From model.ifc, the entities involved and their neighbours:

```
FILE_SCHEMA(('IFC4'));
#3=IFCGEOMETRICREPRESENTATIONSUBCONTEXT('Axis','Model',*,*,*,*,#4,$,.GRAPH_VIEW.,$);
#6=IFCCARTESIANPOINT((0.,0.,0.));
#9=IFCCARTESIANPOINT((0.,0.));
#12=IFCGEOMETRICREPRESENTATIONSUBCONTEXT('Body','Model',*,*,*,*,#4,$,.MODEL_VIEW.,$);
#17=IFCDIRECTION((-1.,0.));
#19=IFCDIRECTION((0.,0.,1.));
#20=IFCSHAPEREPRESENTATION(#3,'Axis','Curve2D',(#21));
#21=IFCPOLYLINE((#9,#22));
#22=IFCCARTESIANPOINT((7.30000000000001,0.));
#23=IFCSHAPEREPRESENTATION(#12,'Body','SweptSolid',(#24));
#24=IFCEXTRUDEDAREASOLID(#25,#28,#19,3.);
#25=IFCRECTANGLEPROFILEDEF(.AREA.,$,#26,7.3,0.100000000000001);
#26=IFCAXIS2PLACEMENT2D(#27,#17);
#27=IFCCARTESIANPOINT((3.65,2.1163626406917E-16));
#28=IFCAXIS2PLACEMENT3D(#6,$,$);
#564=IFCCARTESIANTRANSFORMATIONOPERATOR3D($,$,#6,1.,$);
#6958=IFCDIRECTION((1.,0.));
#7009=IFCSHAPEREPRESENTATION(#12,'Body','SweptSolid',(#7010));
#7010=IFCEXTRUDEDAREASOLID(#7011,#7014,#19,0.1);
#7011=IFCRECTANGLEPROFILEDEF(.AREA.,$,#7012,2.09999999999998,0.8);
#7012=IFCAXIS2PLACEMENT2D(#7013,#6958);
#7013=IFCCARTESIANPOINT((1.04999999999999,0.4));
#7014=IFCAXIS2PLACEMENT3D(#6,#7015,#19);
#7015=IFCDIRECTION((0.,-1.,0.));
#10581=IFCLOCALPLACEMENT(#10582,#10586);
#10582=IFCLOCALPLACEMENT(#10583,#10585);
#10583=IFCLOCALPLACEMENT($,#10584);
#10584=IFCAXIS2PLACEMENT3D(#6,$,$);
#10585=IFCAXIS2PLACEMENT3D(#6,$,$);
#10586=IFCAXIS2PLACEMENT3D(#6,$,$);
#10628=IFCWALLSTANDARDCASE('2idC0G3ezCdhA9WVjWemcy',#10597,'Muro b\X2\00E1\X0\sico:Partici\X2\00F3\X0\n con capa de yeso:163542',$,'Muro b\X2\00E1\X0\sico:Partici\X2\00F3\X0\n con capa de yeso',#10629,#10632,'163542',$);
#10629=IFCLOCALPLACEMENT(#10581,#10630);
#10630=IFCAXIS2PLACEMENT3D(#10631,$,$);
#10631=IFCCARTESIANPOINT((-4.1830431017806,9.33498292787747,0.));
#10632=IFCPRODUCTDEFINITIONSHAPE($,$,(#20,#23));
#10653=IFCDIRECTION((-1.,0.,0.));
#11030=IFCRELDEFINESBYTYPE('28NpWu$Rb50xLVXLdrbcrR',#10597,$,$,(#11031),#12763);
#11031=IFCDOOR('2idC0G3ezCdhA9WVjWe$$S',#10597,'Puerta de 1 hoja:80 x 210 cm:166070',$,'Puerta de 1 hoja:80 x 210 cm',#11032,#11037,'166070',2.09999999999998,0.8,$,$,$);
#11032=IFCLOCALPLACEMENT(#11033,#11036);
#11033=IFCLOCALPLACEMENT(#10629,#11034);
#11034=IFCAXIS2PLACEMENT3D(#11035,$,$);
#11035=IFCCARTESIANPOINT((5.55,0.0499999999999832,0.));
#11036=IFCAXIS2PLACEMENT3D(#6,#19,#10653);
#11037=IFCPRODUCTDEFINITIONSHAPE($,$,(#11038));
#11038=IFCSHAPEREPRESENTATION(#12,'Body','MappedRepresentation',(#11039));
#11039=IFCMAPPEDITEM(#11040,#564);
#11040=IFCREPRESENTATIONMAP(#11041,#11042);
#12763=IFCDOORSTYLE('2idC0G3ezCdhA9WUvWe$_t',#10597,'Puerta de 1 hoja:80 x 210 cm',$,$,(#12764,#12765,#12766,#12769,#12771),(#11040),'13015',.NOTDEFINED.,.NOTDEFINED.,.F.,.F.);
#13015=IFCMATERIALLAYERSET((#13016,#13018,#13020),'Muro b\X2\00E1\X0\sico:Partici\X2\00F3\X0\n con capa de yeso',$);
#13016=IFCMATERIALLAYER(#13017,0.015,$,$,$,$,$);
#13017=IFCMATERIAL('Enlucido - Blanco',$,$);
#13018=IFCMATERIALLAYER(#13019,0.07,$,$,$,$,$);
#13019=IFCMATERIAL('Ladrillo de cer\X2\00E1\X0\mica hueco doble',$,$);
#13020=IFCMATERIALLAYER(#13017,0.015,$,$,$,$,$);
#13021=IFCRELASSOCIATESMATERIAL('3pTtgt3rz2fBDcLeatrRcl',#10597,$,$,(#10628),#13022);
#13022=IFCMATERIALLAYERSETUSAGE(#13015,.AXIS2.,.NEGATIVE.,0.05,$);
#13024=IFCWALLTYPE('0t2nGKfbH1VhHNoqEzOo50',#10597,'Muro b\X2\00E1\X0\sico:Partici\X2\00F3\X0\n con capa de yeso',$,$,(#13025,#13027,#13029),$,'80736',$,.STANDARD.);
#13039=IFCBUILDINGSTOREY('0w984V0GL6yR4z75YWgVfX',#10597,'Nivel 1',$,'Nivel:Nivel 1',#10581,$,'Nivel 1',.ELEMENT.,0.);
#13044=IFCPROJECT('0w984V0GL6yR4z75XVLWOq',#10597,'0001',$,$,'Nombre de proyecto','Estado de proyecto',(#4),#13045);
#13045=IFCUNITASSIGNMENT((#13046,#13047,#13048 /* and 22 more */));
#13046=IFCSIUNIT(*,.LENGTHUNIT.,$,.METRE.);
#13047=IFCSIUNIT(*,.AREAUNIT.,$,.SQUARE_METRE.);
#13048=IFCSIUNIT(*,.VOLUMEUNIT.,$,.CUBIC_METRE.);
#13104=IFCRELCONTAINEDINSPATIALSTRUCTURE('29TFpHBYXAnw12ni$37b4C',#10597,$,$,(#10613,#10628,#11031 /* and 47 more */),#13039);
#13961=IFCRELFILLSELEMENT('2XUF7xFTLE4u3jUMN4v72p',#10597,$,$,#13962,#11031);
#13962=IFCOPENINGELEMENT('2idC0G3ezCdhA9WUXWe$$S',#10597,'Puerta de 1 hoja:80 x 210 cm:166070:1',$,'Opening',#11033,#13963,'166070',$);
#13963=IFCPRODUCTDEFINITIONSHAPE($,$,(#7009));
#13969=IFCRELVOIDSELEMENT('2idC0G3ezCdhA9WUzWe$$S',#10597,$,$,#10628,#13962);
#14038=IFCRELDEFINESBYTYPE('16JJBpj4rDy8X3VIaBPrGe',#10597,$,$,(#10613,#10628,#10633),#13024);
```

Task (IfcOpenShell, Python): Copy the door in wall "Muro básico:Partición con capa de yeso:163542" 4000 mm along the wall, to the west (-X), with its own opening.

```python
import ifcopenshell
import ifcopenshell.api.feature
import ifcopenshell.api.geometry
import ifcopenshell.api.root
import ifcopenshell.geom
import ifcopenshell.util.element
import ifcopenshell.util.placement
import ifcopenshell.util.shape

model = ifcopenshell.open("model.ifc")
settings = ifcopenshell.geom.settings()


def volume(element):
    """Net volume in cubic metres, openings subtracted."""
    shape = ifcopenshell.geom.create_shape(settings, element)
    return ifcopenshell.util.shape.get_volume(shape.geometry)


def reuse_history(source, copy):
    """copy_class also copies each property set's owner history, people and application; keep the originals."""
    for rel in copy.IsDefinedBy:
        if rel.is_a("IfcRelDefinesByProperties") and (history := rel.RelatingPropertyDefinition.OwnerHistory):
            rel.RelatingPropertyDefinition.OwnerHistory = source.OwnerHistory
            ifcopenshell.util.element.remove_deep2(model, history)


door = model.by_guid("2idC0G3ezCdhA9WVjWe$$S")
opening = door.FillsVoids[0].RelatingOpeningElement
wall = opening.VoidsElements[0].RelatingBuildingElement
before = volume(wall)
shift = ifcopenshell.util.placement.get_local_placement(wall.ObjectPlacement)[:3, 0] * -4.0

# copy_class copies the void relationship, type, container and properties, but no geometry.
new_opening = ifcopenshell.api.root.copy_class(model, product=opening)
new_opening.Representation = ifcopenshell.util.element.copy_deep(
    model, opening.Representation, exclude=["IfcGeometricRepresentationContext", "IfcRepresentationMap"]
)
new_opening.Name = "Puerta de 1 hoja:80 x 210 cm"
new_opening.Tag = None
new_door = ifcopenshell.api.root.copy_class(model, product=door)
new_door.Representation = ifcopenshell.util.element.copy_deep(
    model, door.Representation, exclude=["IfcGeometricRepresentationContext", "IfcRepresentationMap"]
)
new_door.Name = "Puerta de 1 hoja:80 x 210 cm"
new_door.Tag = None
reuse_history(door, new_door)
ifcopenshell.api.feature.add_filling(model, opening=new_opening, element=new_door)

for old, new in ((opening, new_opening), (door, new_door)):
    matrix = ifcopenshell.util.placement.get_local_placement(old.ObjectPlacement)
    matrix[:3, 3] += shift
    ifcopenshell.api.geometry.edit_object_placement(model, product=new, matrix=matrix, is_si=False)

after = volume(wall)

print(f"wall volume {before:.3f} -> {after:.3f} m3")

model.write("model-out.ifc")
```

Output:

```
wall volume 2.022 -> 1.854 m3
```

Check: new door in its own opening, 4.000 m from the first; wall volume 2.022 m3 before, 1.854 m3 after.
